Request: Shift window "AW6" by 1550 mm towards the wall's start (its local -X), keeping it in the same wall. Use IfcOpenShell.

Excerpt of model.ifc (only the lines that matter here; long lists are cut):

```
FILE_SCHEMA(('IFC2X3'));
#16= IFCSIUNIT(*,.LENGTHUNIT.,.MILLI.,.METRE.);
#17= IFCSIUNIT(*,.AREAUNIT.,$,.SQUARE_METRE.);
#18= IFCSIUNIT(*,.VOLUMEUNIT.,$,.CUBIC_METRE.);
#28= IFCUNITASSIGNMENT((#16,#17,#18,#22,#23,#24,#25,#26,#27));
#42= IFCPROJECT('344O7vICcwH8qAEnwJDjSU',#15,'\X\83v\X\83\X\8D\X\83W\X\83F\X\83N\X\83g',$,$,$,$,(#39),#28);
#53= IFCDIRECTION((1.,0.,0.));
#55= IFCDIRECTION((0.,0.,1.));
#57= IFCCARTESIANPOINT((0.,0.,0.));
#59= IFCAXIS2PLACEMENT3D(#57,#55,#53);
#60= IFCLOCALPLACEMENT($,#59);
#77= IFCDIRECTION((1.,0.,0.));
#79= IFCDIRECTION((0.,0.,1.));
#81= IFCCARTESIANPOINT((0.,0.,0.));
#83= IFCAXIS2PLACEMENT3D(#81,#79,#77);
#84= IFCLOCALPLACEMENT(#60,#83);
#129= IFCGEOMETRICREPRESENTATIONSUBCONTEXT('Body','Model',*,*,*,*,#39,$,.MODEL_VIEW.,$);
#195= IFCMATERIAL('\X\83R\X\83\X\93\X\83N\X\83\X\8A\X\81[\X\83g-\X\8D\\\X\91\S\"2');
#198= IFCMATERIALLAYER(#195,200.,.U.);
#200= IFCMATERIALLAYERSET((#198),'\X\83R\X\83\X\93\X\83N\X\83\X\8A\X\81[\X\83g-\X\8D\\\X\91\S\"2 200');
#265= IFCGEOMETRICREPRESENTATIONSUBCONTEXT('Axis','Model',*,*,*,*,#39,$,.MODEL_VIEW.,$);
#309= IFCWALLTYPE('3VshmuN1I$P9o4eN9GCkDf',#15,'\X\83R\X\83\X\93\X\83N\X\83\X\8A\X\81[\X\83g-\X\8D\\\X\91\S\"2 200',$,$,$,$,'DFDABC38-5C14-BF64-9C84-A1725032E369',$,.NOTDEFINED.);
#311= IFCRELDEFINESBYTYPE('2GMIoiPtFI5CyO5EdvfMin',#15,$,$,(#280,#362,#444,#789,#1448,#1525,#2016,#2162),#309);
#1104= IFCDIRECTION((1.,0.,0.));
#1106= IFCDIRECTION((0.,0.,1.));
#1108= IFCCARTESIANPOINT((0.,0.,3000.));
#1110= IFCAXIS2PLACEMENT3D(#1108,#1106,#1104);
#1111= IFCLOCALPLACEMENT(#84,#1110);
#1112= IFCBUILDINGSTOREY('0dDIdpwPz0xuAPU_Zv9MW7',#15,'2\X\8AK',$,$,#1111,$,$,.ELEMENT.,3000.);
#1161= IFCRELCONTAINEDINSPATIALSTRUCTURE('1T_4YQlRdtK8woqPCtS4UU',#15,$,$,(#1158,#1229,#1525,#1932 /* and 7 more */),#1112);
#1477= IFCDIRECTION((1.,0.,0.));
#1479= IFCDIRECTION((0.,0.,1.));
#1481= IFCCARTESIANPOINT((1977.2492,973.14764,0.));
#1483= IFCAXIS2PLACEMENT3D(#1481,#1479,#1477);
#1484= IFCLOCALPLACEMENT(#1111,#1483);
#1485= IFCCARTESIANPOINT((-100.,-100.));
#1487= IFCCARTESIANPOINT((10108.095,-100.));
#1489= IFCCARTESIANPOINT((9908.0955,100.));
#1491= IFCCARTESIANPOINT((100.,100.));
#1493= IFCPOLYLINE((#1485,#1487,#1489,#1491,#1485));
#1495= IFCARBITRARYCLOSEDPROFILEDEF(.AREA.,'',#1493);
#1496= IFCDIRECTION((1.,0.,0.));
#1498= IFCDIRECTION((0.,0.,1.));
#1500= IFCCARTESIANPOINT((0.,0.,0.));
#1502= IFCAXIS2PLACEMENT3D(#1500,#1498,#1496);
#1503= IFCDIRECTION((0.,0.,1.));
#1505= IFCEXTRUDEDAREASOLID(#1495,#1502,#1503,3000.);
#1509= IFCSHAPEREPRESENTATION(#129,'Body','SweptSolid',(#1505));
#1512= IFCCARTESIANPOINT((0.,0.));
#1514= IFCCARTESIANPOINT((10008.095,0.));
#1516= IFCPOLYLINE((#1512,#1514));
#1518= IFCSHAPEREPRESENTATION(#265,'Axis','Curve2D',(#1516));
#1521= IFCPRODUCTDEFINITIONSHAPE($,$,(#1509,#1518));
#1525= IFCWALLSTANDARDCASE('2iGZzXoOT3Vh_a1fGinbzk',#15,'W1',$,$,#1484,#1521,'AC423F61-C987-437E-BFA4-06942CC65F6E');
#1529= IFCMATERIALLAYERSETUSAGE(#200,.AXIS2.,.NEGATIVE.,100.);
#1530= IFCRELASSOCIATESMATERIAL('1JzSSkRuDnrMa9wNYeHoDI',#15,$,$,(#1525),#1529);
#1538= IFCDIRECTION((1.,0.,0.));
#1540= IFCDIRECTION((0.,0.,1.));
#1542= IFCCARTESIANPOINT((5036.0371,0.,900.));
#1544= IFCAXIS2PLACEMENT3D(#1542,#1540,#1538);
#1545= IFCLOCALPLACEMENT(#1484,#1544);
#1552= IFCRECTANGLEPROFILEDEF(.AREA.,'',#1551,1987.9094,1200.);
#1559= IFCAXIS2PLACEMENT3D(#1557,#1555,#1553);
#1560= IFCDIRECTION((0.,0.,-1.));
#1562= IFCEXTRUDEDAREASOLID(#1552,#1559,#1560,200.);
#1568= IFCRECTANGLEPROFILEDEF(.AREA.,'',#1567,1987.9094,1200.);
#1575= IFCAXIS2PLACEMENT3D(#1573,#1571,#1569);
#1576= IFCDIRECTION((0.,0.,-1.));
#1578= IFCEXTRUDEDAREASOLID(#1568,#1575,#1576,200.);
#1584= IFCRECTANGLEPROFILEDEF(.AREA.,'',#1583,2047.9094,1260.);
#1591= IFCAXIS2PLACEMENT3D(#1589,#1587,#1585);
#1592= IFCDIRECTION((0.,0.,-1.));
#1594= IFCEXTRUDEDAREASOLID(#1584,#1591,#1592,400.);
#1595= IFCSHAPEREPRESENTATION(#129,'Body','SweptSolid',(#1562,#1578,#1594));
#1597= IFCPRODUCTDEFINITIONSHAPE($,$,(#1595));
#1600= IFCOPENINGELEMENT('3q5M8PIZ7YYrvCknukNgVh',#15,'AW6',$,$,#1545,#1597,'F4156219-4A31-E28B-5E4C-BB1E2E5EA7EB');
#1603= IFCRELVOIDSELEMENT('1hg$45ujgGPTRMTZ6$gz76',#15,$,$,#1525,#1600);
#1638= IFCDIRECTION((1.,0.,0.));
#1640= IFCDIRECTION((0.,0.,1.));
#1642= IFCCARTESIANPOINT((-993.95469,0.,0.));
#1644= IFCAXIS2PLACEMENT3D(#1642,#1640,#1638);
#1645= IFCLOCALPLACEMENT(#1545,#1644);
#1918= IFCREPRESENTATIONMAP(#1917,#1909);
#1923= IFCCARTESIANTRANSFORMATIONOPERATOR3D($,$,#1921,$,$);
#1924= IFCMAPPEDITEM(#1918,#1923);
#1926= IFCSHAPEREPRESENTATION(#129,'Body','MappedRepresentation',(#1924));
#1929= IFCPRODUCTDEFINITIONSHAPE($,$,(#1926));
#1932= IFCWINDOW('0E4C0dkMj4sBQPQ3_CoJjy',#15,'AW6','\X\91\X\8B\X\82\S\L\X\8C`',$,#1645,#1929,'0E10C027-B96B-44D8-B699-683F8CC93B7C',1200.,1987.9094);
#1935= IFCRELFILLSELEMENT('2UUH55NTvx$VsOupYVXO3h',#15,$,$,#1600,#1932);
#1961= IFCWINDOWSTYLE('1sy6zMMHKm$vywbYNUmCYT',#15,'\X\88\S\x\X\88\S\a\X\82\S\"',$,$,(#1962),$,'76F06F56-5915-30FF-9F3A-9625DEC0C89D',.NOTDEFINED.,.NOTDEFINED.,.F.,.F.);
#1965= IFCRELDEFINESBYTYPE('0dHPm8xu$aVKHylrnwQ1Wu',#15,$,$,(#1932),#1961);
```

```python
import ifcopenshell
import ifcopenshell.api.geometry
import ifcopenshell.util.placement

model = ifcopenshell.open("model.ifc")

window = model.by_guid("0E4C0dkMj4sBQPQ3_CoJjy")
opening = window.FillsVoids[0].RelatingOpeningElement
wall = opening.VoidsElements[0].RelatingBuildingElement

wall_matrix = ifcopenshell.util.placement.get_local_placement(wall.ObjectPlacement)
shift = wall_matrix[:3, 0] * -1550.0
before = ifcopenshell.util.placement.get_local_placement(window.ObjectPlacement)[:3, 3].copy()

# The window is placed relative to its opening, so it follows when the opening moves.
matrix = ifcopenshell.util.placement.get_local_placement(opening.ObjectPlacement)
matrix[:3, 3] += shift
ifcopenshell.api.geometry.edit_object_placement(
    model, product=opening, matrix=matrix, is_si=False, should_transform_children=True
)

after = ifcopenshell.util.placement.get_local_placement(window.ObjectPlacement)[:3, 3]
print("window moved by", (after - before).round(3) + 0.0)

model.write("model_updated.ifc")
```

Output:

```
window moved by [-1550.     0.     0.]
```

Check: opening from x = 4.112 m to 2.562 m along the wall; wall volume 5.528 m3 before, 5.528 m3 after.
